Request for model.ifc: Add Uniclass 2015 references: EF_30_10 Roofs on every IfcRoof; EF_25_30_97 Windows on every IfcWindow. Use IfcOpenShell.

First a look at what the model holds.

```python
import ifcopenshell

model = ifcopenshell.open("model.ifc")
print(model.schema)
print("classifications:", [c.Name for c in model.by_type("IfcClassification")])
for ifc_class in ("IfcDoor", "IfcRoof", "IfcStair", "IfcWall", "IfcWindow"):
    print(ifc_class, len(model.by_type(ifc_class)))
```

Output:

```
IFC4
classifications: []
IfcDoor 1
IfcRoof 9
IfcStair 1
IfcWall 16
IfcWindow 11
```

```python
import ifcopenshell
import ifcopenshell.api.classification

model = ifcopenshell.open("model.ifc")

system = ifcopenshell.api.classification.add_classification(model, classification="Uniclass 2015")

codes = {
    "IfcRoof": ("EF_30_10", "Roofs"),
    "IfcWindow": ("EF_25_30_97", "Windows"),
}
for ifc_class, (code, name) in codes.items():
    products = model.by_type(ifc_class)
    ifcopenshell.api.classification.add_reference(
        model, products=products, classification=system, identification=code, name=name
    )
    print(code, len(products))

model.write("model-out.ifc")
```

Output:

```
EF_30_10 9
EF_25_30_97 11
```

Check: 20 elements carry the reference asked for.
